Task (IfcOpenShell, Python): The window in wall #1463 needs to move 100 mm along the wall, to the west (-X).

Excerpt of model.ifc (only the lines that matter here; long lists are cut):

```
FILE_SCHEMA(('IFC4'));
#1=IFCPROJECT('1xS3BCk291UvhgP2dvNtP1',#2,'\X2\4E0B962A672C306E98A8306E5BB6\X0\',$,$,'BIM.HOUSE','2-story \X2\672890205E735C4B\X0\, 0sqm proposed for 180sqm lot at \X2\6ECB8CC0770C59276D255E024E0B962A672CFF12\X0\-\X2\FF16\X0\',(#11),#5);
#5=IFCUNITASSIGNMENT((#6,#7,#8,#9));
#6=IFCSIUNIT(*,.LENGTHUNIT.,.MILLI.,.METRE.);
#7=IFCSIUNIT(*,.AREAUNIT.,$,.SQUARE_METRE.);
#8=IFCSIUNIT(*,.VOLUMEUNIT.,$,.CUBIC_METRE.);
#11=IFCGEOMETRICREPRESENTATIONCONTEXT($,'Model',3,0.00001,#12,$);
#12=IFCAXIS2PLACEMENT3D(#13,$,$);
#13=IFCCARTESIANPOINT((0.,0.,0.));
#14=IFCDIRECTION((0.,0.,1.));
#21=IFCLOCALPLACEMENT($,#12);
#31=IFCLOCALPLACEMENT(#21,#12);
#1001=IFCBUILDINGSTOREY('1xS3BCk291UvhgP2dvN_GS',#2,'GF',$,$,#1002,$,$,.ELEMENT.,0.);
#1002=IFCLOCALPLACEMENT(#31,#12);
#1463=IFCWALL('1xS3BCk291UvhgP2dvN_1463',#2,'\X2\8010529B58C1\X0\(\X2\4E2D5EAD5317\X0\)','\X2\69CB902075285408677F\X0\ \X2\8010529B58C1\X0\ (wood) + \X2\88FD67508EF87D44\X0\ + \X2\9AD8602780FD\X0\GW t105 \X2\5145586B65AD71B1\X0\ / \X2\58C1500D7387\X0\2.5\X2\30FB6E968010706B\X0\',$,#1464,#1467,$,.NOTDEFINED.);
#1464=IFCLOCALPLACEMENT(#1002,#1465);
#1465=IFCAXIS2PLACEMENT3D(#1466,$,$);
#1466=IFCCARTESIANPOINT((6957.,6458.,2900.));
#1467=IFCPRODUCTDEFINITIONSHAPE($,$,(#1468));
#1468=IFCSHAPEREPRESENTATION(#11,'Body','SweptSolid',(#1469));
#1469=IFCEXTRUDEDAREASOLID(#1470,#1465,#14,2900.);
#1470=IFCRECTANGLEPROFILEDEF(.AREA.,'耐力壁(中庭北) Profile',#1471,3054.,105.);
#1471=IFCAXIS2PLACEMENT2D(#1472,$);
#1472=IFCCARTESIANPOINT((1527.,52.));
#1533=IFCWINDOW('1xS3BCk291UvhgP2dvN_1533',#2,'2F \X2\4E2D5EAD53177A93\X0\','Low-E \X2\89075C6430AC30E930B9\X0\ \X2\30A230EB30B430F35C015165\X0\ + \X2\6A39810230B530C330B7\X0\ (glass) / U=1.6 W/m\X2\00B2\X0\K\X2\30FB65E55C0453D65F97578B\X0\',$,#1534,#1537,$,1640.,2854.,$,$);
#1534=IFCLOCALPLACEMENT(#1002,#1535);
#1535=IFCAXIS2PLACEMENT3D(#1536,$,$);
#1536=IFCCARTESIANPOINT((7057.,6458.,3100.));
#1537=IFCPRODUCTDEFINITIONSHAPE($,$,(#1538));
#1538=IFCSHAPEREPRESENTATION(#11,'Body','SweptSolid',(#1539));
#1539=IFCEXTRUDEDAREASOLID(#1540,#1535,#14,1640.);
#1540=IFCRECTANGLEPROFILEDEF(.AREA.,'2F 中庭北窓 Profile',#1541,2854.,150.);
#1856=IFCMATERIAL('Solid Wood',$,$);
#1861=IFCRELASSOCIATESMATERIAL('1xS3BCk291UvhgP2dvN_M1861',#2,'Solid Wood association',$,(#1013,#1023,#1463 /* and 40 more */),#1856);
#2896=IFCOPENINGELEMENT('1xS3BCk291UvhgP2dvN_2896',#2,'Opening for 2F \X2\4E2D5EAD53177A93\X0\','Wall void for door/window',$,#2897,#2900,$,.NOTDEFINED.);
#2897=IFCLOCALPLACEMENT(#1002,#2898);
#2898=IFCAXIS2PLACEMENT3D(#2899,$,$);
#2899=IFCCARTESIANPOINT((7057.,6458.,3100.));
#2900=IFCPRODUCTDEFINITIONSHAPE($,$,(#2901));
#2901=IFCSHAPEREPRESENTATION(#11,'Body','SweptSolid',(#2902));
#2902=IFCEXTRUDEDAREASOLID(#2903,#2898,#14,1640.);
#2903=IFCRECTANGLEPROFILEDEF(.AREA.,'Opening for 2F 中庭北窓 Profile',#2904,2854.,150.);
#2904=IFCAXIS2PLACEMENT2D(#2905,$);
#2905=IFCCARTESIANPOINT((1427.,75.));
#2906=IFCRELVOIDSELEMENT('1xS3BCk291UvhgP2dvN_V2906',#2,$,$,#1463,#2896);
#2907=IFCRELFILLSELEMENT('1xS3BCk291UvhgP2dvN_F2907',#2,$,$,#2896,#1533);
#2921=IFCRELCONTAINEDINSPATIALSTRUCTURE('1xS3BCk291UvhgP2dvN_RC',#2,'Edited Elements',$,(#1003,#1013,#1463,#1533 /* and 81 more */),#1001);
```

```python
import ifcopenshell
import ifcopenshell.api.geometry
import ifcopenshell.util.placement

model = ifcopenshell.open("model.ifc")

window = model.by_id(1533)
opening = window.FillsVoids[0].RelatingOpeningElement
wall = opening.VoidsElements[0].RelatingBuildingElement

wall_matrix = ifcopenshell.util.placement.get_local_placement(wall.ObjectPlacement)
shift = wall_matrix[:3, 0] * -100.0
before = ifcopenshell.util.placement.get_local_placement(window.ObjectPlacement)[:3, 3].copy()

# The window is not placed relative to its opening, so move both.
for product in (opening, window):
    matrix = ifcopenshell.util.placement.get_local_placement(product.ObjectPlacement)
    matrix[:3, 3] += shift
    ifcopenshell.api.geometry.edit_object_placement(model, product=product, matrix=matrix, is_si=False)

after = ifcopenshell.util.placement.get_local_placement(window.ObjectPlacement)[:3, 3]
print("window moved by", (after - before).round(3) + 0.0)

model.write("model_edited.ifc")
```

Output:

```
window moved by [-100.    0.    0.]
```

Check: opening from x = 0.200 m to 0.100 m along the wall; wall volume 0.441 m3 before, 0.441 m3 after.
